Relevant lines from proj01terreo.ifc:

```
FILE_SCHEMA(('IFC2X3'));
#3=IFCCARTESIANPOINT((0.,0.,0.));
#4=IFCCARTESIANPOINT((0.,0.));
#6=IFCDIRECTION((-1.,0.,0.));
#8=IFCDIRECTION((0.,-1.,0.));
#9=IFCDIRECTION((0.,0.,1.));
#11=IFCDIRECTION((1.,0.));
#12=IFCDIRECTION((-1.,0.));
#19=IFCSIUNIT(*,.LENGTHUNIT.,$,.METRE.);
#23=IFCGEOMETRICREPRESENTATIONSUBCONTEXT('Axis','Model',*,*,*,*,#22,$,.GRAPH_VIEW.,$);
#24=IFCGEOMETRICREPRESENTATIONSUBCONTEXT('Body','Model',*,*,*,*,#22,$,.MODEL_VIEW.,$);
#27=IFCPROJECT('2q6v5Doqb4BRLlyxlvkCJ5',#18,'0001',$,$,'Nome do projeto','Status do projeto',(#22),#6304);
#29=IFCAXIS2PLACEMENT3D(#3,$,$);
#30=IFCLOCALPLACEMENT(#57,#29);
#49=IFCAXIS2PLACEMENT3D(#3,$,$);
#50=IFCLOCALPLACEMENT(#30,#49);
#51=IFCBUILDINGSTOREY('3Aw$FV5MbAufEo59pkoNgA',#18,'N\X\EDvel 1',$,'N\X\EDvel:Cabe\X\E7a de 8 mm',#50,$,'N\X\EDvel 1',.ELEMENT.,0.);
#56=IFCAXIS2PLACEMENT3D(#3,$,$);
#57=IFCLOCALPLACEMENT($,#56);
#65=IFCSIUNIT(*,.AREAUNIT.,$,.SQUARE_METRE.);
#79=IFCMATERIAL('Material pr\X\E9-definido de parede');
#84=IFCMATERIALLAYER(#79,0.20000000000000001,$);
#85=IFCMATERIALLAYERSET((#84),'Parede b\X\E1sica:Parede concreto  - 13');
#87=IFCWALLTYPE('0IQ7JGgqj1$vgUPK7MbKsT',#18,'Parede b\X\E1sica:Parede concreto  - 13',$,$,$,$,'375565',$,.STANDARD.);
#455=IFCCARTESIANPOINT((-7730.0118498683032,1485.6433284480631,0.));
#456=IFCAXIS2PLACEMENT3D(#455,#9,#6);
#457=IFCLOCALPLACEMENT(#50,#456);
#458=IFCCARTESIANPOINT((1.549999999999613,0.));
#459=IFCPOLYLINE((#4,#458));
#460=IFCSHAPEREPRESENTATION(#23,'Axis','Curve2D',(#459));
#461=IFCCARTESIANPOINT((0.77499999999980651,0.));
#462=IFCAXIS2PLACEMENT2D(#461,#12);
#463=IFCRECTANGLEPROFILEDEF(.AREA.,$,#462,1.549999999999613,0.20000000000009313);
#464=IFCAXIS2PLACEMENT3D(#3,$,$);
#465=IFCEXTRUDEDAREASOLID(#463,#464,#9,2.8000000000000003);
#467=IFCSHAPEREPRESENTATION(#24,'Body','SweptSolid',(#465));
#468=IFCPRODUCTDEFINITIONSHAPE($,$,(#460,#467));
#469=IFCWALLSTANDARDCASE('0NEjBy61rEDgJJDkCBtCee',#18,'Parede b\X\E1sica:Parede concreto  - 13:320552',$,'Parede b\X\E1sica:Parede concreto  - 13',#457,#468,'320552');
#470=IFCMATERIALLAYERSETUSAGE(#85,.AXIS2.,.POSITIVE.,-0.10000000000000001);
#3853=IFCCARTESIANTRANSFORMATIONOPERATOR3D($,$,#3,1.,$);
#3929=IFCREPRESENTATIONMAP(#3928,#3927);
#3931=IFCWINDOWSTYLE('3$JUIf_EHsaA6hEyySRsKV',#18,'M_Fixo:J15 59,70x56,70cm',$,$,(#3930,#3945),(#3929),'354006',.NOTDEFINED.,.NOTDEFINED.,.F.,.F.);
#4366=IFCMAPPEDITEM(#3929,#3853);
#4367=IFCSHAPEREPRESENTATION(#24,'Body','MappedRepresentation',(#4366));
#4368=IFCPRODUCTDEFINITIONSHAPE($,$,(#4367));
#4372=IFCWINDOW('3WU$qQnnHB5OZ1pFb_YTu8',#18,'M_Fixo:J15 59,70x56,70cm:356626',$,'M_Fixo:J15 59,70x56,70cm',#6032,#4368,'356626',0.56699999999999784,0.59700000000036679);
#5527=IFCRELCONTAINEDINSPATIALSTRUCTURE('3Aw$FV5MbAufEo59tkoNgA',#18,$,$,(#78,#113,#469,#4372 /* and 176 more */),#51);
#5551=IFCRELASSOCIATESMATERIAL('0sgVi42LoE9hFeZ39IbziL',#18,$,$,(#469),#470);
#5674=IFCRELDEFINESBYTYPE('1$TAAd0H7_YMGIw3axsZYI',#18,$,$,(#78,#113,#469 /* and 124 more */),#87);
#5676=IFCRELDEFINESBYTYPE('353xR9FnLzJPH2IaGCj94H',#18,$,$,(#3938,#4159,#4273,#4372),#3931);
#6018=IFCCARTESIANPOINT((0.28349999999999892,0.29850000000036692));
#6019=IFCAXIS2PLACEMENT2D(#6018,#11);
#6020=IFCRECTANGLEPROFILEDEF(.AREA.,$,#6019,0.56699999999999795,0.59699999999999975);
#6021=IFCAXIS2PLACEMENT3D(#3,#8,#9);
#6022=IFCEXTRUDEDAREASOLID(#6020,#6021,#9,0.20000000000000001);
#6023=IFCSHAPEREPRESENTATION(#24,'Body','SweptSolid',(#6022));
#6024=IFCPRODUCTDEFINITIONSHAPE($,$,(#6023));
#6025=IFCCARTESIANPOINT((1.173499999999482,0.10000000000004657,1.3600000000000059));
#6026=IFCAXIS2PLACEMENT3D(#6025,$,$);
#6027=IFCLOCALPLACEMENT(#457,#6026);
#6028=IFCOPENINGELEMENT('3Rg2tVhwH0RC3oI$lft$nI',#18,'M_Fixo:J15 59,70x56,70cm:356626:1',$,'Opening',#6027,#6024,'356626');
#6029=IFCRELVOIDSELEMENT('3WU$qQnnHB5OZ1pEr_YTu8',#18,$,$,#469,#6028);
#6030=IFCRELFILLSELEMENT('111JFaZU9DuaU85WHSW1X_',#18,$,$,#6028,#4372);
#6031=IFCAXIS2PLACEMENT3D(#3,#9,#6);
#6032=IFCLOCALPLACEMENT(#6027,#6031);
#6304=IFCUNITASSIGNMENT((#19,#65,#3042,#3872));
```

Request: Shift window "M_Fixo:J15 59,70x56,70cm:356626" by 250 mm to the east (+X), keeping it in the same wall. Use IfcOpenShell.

```python
import ifcopenshell
import ifcopenshell.api.geometry
import ifcopenshell.util.placement
import ifcopenshell.util.unit

model = ifcopenshell.open("proj01terreo.ifc")
unit_scale = ifcopenshell.util.unit.calculate_unit_scale(model)

window = model.by_id(4372)
opening = window.FillsVoids[0].RelatingOpeningElement
wall = opening.VoidsElements[0].RelatingBuildingElement

wall_matrix = ifcopenshell.util.placement.get_local_placement(wall.ObjectPlacement)
shift = wall_matrix[:3, 0] * -0.25 / unit_scale
before = ifcopenshell.util.placement.get_local_placement(window.ObjectPlacement)[:3, 3].copy()

# The window is placed relative to its opening, so it follows when the opening moves.
matrix = ifcopenshell.util.placement.get_local_placement(opening.ObjectPlacement)
matrix[:3, 3] += shift
ifcopenshell.api.geometry.edit_object_placement(
    model, product=opening, matrix=matrix, is_si=False, should_transform_children=True
)

after = ifcopenshell.util.placement.get_local_placement(window.ObjectPlacement)[:3, 3]
print("window moved by", (after - before).round(3) + 0.0)

model.write("proj01terreo_updated.ifc")
```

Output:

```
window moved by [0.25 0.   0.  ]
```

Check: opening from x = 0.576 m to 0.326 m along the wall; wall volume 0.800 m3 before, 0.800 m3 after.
